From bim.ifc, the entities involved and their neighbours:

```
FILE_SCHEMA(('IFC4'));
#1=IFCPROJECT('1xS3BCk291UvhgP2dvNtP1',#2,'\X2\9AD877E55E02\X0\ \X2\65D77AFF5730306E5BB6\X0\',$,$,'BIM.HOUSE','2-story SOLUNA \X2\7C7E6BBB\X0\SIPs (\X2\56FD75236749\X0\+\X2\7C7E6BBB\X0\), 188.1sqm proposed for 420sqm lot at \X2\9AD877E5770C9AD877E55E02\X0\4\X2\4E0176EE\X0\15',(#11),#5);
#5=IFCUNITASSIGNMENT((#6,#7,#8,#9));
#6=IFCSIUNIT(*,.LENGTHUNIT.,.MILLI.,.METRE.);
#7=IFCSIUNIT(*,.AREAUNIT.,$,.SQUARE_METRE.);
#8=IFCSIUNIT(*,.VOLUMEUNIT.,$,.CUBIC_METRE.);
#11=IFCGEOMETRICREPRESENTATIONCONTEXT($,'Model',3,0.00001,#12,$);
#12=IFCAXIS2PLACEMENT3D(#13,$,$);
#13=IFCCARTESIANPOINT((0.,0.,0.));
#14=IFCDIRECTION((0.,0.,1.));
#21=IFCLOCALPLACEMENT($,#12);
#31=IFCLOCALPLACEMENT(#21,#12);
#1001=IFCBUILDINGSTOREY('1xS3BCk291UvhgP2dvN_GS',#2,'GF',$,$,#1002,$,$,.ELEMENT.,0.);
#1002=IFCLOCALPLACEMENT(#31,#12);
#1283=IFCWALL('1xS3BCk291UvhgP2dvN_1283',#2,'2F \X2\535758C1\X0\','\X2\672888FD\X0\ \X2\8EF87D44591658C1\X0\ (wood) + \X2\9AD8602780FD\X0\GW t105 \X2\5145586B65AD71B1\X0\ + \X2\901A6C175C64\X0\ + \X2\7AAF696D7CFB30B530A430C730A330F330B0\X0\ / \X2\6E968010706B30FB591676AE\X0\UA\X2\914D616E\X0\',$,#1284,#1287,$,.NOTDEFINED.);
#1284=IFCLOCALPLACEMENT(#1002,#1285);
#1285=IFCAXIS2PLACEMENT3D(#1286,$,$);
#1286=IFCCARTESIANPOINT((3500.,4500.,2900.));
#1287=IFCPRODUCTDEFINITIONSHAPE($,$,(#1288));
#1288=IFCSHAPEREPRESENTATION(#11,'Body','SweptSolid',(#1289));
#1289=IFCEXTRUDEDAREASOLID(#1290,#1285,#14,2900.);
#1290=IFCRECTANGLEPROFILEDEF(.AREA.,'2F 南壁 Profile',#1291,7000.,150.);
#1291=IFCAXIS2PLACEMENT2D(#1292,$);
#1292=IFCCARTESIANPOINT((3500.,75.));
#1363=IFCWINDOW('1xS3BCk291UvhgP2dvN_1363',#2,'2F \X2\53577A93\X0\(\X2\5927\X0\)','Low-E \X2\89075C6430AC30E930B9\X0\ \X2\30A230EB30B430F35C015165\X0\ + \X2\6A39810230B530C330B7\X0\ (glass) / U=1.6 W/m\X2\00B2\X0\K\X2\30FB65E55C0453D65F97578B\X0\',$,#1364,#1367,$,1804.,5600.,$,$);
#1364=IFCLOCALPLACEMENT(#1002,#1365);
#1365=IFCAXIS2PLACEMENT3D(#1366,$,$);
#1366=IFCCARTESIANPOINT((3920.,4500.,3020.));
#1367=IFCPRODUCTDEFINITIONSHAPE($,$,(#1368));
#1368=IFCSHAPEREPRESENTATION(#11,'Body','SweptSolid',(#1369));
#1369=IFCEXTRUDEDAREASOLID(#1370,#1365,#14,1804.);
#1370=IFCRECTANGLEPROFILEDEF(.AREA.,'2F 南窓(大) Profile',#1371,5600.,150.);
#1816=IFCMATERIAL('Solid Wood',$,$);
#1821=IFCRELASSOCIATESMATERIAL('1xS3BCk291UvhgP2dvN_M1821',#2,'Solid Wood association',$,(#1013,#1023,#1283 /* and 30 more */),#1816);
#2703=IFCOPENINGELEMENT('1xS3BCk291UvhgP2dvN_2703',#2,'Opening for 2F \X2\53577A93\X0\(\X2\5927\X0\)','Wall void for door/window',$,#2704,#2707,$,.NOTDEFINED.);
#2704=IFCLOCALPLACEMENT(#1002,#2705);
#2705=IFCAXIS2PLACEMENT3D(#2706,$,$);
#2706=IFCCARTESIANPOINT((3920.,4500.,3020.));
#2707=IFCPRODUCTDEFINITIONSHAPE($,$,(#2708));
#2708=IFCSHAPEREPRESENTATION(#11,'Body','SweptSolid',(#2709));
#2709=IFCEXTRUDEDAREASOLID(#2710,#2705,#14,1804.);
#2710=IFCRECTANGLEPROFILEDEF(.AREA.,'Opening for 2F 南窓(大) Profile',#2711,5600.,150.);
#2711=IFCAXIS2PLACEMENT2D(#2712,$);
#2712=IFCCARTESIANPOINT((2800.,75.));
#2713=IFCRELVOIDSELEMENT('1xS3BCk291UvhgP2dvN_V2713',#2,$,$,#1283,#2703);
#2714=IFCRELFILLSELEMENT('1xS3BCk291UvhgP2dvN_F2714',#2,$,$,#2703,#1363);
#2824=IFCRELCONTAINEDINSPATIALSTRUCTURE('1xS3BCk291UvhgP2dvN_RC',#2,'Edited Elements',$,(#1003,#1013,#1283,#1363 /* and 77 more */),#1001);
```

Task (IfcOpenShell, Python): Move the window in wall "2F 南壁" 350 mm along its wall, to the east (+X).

```python
import ifcopenshell
import ifcopenshell.api.geometry
import ifcopenshell.util.placement
import ifcopenshell.util.unit

model = ifcopenshell.open("bim.ifc")
unit_scale = ifcopenshell.util.unit.calculate_unit_scale(model)

window = model.by_guid("1xS3BCk291UvhgP2dvN_1363")
opening = window.FillsVoids[0].RelatingOpeningElement
wall = opening.VoidsElements[0].RelatingBuildingElement

wall_matrix = ifcopenshell.util.placement.get_local_placement(wall.ObjectPlacement)
shift = wall_matrix[:3, 0] * 0.35 / unit_scale
before = ifcopenshell.util.placement.get_local_placement(window.ObjectPlacement)[:3, 3].copy()

# The window is not placed relative to its opening, so move both.
for product in (opening, window):
    matrix = ifcopenshell.util.placement.get_local_placement(product.ObjectPlacement)
    matrix[:3, 3] += shift
    ifcopenshell.api.geometry.edit_object_placement(model, product=product, matrix=matrix, is_si=False)

after = ifcopenshell.util.placement.get_local_placement(window.ObjectPlacement)[:3, 3]
print("window moved by", (after - before).round(3) + 0.0)

model.write("bim_v2.ifc")
```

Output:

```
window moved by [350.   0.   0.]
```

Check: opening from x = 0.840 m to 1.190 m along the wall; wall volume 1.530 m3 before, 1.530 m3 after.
